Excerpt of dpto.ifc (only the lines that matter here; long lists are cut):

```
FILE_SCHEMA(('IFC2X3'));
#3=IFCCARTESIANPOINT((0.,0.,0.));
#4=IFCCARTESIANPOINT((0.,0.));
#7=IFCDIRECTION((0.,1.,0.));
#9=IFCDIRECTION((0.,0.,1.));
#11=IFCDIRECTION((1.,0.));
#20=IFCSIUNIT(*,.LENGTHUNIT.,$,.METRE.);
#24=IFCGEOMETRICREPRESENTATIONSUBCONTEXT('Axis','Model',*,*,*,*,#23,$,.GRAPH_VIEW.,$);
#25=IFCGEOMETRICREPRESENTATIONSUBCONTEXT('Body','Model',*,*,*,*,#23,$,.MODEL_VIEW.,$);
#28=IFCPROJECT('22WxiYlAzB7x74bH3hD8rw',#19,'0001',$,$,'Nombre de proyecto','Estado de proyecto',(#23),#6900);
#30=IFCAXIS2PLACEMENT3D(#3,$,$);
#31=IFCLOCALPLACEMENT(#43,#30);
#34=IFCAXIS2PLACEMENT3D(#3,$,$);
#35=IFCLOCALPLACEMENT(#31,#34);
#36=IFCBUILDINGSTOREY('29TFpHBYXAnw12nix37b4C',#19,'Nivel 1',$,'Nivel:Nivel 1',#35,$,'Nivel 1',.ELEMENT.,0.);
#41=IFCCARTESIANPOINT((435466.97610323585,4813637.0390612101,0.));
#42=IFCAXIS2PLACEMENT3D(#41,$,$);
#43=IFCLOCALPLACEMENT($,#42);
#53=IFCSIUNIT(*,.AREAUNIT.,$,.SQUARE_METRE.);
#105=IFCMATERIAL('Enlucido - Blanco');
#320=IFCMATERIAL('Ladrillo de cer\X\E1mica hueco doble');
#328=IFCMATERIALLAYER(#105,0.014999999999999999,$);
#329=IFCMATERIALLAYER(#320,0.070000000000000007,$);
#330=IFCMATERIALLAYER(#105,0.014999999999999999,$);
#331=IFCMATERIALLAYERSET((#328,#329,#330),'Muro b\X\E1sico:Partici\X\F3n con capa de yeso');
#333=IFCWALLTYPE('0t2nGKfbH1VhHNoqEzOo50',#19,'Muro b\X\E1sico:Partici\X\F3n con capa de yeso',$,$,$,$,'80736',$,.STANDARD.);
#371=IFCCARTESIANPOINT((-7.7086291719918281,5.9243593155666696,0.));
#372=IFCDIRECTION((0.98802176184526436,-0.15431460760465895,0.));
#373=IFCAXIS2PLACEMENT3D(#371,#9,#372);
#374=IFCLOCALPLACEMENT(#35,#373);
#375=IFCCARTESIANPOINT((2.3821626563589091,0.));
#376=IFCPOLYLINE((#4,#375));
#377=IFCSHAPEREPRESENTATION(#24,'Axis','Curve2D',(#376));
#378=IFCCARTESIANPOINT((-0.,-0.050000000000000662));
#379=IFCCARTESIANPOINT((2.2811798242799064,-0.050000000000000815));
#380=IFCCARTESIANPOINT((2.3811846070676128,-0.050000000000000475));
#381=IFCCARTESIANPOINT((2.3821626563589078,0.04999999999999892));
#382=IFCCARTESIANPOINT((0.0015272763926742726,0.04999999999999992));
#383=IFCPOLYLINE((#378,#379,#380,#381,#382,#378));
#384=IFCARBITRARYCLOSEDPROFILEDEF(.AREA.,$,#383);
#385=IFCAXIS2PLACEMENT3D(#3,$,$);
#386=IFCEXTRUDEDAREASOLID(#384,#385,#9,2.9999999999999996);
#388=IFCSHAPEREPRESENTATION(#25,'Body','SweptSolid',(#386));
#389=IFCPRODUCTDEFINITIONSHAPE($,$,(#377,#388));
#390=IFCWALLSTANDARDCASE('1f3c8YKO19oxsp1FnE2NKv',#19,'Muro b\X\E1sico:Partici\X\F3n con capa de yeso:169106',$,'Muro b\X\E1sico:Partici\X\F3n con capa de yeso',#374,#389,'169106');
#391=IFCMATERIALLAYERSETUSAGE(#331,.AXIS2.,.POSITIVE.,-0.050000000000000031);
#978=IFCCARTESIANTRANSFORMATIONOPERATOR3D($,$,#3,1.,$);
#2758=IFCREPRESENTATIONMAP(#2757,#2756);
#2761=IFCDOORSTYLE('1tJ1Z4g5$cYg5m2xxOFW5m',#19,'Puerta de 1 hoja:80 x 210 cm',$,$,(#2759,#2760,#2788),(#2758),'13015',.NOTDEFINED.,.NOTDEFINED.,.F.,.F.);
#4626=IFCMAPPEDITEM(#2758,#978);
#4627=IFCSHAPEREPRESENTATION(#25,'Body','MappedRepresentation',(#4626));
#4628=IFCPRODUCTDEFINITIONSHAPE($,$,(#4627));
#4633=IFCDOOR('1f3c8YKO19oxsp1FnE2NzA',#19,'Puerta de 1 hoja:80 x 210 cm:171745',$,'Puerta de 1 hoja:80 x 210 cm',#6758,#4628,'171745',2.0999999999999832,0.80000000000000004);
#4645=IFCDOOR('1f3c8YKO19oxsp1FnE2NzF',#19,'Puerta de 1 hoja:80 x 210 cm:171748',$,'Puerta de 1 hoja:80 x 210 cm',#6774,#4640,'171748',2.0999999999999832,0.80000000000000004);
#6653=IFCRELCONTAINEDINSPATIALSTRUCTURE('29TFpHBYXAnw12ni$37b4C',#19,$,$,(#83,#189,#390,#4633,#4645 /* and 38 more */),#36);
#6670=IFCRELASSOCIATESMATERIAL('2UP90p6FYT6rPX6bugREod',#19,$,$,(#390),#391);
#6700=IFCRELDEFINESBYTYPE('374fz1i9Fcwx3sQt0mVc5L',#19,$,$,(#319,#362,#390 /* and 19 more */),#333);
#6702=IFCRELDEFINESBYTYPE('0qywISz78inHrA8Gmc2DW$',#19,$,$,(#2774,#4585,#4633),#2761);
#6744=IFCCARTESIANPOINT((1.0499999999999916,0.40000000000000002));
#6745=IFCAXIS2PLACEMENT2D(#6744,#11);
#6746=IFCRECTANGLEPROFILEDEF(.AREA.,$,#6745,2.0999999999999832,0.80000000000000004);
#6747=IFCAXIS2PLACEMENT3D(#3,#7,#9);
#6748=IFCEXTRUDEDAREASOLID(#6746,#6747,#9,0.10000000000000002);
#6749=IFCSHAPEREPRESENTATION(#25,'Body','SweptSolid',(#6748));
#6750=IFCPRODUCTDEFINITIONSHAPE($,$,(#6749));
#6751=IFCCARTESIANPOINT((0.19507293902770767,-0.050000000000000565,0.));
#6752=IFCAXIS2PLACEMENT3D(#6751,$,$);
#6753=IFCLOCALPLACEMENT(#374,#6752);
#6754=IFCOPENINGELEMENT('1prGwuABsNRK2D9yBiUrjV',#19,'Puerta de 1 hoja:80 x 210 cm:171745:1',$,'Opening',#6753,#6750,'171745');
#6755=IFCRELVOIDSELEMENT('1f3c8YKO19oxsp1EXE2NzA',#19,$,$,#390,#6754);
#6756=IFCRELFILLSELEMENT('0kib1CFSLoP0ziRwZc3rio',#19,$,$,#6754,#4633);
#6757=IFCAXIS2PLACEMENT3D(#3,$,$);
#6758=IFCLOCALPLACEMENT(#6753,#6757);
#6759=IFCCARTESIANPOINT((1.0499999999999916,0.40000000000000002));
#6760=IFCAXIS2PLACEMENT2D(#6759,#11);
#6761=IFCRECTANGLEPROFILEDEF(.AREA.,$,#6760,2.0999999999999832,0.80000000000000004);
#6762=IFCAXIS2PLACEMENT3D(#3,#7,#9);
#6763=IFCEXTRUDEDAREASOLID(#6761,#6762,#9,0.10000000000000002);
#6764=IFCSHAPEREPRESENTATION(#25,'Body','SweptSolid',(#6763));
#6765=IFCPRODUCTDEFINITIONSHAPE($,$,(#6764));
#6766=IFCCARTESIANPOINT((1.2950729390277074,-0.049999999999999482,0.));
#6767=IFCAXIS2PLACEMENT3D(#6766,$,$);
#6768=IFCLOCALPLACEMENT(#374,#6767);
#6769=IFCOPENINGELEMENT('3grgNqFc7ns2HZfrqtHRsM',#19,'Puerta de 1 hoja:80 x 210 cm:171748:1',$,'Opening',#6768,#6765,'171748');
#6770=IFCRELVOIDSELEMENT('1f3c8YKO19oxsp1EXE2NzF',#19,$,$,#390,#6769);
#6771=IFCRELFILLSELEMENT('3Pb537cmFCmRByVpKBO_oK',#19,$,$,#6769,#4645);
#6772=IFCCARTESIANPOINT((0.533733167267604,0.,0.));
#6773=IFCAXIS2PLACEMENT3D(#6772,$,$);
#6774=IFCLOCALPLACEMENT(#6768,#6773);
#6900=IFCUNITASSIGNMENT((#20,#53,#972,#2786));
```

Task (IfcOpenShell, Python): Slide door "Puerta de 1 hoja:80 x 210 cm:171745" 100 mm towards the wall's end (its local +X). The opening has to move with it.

```python
import ifcopenshell
import ifcopenshell.api.geometry
import ifcopenshell.util.placement
import ifcopenshell.util.unit

model = ifcopenshell.open("dpto.ifc")
unit_scale = ifcopenshell.util.unit.calculate_unit_scale(model)

door = model.by_guid("1f3c8YKO19oxsp1FnE2NzA")
opening = door.FillsVoids[0].RelatingOpeningElement
wall = opening.VoidsElements[0].RelatingBuildingElement

wall_matrix = ifcopenshell.util.placement.get_local_placement(wall.ObjectPlacement)
shift = wall_matrix[:3, 0] * 0.1 / unit_scale
before = ifcopenshell.util.placement.get_local_placement(door.ObjectPlacement)[:3, 3].copy()

# The door is placed relative to its opening, so it follows when the opening moves.
matrix = ifcopenshell.util.placement.get_local_placement(opening.ObjectPlacement)
matrix[:3, 3] += shift
ifcopenshell.api.geometry.edit_object_placement(
    model, product=opening, matrix=matrix, is_si=False, should_transform_children=True
)

after = ifcopenshell.util.placement.get_local_placement(door.ObjectPlacement)[:3, 3]
print("door moved by", (after - before).round(3) + 0.0)

model.write("dpto_v2.ifc")
```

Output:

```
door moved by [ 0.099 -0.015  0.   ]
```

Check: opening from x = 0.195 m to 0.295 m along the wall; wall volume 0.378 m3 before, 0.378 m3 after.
